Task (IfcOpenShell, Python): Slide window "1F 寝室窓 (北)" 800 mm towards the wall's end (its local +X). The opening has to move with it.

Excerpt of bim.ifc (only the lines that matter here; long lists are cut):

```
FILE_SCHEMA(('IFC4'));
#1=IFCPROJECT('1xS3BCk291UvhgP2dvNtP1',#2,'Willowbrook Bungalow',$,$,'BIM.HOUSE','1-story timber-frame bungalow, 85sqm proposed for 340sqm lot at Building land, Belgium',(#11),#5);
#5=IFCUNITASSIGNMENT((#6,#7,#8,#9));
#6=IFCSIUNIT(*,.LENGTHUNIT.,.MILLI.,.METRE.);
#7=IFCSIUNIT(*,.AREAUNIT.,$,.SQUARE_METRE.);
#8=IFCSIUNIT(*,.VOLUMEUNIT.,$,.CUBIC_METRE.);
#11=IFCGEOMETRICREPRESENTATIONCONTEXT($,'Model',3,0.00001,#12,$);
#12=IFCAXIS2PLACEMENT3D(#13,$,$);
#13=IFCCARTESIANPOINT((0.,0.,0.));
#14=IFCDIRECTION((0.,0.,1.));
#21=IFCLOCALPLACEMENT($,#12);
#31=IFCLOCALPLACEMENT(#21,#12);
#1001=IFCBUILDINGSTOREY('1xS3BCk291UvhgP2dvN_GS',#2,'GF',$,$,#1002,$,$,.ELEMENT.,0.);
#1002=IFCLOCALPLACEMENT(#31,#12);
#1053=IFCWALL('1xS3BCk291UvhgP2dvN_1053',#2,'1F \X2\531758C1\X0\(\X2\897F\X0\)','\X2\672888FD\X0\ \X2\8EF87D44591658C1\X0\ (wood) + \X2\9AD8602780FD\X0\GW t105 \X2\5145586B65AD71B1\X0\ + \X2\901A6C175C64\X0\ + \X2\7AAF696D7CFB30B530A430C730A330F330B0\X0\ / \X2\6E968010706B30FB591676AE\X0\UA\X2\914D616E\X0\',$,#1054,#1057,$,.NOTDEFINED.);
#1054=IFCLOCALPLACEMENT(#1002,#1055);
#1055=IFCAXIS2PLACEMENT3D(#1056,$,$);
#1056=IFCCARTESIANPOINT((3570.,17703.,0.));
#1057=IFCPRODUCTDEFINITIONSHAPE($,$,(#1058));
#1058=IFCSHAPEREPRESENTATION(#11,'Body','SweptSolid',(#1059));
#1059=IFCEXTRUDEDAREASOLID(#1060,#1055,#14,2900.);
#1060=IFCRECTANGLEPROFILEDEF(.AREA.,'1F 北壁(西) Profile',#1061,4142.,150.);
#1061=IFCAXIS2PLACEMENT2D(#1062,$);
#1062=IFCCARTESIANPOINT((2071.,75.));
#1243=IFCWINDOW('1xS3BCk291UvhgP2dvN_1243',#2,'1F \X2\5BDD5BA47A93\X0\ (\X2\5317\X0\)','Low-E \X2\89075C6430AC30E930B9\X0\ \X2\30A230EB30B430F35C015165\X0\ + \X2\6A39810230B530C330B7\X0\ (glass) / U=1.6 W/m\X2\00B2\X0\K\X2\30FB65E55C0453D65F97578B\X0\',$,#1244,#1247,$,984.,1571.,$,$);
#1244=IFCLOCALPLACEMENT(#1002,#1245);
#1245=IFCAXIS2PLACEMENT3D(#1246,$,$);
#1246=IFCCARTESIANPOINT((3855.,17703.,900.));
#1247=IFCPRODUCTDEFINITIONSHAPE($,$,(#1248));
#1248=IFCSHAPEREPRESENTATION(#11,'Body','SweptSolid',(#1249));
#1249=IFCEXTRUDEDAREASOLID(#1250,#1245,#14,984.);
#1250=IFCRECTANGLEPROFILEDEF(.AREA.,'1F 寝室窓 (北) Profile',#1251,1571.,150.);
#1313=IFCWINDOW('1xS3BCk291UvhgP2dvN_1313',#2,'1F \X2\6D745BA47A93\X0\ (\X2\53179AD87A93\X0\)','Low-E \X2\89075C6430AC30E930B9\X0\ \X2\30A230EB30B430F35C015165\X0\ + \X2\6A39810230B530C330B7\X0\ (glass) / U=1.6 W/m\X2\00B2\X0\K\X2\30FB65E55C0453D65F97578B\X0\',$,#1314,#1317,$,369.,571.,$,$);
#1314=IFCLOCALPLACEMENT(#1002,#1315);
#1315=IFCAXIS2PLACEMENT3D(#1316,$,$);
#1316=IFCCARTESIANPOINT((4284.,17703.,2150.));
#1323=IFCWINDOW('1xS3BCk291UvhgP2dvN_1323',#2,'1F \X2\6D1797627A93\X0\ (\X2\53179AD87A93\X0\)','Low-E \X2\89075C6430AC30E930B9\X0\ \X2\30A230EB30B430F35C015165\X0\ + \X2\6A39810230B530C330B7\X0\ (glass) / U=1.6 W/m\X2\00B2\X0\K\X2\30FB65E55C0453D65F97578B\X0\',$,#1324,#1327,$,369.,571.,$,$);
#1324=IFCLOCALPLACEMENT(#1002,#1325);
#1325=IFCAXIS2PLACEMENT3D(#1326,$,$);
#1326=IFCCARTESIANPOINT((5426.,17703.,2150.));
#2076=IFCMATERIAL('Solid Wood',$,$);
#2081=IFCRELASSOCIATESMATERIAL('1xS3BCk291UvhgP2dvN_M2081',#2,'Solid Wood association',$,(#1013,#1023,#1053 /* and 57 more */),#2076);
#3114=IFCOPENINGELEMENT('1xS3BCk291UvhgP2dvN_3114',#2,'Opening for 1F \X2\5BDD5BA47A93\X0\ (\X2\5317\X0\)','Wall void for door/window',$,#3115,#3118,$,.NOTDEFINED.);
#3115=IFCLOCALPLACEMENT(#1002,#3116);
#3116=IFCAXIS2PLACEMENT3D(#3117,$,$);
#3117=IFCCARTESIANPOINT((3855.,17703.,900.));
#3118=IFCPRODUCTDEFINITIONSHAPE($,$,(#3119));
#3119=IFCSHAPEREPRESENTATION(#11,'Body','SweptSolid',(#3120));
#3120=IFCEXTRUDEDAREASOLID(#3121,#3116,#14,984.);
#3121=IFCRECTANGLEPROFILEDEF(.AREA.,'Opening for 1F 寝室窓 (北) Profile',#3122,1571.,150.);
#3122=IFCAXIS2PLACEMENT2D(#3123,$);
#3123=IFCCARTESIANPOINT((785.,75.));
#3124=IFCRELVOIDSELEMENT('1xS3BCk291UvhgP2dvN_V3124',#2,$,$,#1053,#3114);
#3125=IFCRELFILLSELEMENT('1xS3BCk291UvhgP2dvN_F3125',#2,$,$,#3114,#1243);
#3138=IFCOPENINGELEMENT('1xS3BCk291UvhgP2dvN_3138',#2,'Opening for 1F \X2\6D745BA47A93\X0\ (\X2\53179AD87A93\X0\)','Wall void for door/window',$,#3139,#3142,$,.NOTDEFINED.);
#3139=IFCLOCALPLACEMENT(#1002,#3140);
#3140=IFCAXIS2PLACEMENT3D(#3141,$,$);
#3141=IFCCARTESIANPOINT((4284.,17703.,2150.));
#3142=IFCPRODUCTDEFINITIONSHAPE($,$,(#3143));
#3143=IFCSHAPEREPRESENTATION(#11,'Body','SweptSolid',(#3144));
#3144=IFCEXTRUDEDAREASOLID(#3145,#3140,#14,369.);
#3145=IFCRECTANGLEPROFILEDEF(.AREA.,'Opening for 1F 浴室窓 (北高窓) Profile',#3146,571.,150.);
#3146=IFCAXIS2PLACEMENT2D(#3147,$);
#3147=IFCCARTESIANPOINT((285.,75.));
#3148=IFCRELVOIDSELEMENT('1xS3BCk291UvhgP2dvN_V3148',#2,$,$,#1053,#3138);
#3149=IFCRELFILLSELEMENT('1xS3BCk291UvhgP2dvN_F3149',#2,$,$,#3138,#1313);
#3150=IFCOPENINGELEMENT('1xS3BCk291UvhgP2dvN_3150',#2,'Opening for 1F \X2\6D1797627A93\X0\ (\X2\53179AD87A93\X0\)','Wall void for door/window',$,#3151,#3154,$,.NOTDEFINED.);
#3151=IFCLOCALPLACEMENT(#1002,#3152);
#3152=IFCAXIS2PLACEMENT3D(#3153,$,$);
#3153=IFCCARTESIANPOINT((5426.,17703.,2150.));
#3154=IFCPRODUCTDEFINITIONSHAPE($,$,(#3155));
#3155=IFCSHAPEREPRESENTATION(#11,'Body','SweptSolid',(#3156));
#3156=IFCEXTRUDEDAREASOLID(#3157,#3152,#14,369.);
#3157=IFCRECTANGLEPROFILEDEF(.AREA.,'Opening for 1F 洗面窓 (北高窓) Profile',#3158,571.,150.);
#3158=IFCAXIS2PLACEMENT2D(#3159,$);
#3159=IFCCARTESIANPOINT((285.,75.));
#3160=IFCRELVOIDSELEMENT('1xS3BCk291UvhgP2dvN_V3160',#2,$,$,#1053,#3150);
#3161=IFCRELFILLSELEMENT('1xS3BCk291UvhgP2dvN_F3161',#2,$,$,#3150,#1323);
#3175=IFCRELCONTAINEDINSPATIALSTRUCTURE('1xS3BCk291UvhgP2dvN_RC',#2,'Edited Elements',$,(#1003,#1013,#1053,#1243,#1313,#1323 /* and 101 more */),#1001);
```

```python
import ifcopenshell
import ifcopenshell.api.geometry
import ifcopenshell.util.placement

model = ifcopenshell.open("bim.ifc")

window = model.by_id(1243)
opening = window.FillsVoids[0].RelatingOpeningElement
wall = opening.VoidsElements[0].RelatingBuildingElement

wall_matrix = ifcopenshell.util.placement.get_local_placement(wall.ObjectPlacement)
shift = wall_matrix[:3, 0] * 800.0
before = ifcopenshell.util.placement.get_local_placement(window.ObjectPlacement)[:3, 3].copy()

# The window is not placed relative to its opening, so move both.
for product in (opening, window):
    matrix = ifcopenshell.util.placement.get_local_placement(product.ObjectPlacement)
    matrix[:3, 3] += shift
    ifcopenshell.api.geometry.edit_object_placement(model, product=product, matrix=matrix, is_si=False)

after = ifcopenshell.util.placement.get_local_placement(window.ObjectPlacement)[:3, 3]
print("window moved by", (after - before).round(3) + 0.0)

model.write("bim_rev.ifc")
```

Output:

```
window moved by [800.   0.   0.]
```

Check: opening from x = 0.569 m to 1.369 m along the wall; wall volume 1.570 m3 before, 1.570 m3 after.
